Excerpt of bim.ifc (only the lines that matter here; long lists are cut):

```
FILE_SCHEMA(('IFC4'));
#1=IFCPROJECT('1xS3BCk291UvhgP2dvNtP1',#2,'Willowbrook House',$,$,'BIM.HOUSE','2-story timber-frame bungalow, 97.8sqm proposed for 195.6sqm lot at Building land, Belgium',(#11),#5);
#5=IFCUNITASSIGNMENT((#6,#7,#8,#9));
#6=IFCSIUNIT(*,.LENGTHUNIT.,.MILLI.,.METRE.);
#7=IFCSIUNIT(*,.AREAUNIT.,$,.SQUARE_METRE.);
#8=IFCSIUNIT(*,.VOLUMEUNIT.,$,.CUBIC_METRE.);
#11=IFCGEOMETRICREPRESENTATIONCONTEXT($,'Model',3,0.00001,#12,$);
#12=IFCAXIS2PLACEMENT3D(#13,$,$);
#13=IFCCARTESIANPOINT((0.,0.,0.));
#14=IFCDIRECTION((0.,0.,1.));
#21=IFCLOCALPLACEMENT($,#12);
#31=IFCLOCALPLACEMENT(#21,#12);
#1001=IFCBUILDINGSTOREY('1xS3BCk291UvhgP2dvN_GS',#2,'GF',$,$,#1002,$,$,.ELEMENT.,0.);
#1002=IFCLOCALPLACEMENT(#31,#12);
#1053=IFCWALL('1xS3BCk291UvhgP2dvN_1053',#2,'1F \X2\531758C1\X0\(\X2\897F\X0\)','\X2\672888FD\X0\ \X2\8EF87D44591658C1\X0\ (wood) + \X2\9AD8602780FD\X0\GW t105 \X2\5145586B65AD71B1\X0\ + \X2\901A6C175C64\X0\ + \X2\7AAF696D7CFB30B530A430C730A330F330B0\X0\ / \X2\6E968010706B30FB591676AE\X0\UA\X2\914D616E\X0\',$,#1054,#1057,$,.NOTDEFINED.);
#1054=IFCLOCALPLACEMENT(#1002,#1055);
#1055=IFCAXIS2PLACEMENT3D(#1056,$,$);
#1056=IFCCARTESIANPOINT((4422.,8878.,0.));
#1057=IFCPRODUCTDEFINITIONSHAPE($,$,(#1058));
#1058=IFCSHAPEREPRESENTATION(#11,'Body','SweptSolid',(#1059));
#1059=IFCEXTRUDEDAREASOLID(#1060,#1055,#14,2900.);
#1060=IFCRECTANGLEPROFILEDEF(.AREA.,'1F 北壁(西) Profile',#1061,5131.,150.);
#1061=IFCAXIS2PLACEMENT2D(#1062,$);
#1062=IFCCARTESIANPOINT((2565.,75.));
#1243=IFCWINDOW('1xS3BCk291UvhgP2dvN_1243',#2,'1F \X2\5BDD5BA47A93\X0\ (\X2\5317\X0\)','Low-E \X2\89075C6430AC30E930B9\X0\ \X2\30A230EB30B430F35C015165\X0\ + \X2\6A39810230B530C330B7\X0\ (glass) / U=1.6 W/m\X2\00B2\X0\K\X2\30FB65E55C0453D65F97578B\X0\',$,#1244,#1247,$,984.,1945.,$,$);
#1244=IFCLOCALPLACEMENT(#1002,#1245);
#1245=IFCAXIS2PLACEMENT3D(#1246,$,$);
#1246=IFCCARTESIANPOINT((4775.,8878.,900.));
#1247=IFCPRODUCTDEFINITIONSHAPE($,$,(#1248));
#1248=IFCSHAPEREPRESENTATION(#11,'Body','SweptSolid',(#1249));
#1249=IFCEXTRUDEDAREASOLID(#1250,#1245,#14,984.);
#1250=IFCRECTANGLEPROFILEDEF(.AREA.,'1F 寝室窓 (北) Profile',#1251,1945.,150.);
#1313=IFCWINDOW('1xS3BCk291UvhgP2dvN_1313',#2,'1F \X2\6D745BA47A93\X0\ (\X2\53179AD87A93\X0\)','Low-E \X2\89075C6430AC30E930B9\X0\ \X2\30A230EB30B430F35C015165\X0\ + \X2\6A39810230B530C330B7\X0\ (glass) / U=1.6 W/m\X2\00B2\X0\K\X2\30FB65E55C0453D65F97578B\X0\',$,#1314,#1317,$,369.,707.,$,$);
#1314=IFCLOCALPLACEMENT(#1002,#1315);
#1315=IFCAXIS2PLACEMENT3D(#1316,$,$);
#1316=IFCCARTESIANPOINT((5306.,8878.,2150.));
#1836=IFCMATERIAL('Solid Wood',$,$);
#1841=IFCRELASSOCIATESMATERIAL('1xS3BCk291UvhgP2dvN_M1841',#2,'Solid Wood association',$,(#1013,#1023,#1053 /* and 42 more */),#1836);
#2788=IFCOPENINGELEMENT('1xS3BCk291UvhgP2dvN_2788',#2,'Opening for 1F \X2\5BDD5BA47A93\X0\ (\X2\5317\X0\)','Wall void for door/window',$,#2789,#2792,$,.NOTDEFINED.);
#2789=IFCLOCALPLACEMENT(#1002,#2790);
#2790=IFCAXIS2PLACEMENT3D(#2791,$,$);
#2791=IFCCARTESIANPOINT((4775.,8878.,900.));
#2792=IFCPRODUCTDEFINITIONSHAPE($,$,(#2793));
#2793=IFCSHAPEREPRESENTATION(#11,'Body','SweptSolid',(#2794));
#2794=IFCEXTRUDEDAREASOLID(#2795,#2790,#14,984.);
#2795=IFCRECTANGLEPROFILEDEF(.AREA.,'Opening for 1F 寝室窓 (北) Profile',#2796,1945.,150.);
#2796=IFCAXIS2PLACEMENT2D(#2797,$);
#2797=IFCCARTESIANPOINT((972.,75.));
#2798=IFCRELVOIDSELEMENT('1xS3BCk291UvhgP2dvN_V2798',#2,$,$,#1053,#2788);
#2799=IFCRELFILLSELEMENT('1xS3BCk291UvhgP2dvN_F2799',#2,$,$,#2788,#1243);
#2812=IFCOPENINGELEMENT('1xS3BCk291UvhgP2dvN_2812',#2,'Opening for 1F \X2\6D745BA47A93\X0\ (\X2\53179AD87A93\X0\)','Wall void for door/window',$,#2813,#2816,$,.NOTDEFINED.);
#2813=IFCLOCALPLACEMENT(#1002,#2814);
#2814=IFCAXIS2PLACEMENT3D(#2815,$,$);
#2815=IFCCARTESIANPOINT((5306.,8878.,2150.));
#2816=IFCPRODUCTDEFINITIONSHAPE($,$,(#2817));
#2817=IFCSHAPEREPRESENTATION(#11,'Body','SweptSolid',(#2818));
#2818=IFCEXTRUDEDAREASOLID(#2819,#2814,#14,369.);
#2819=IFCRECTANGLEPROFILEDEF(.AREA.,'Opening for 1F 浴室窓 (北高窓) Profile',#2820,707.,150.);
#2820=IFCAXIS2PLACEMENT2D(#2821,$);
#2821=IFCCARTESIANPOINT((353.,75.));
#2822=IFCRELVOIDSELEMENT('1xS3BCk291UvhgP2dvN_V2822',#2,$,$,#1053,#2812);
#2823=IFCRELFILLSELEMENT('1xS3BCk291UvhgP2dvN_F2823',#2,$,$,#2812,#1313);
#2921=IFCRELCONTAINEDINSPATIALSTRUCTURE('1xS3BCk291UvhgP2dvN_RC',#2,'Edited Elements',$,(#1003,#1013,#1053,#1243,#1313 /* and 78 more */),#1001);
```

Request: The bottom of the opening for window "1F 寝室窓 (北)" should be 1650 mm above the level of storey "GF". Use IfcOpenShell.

```python
import numpy as np
import ifcopenshell
import ifcopenshell.api.geometry
import ifcopenshell.geom
import ifcopenshell.util.element
import ifcopenshell.util.placement
import ifcopenshell.util.shape
import ifcopenshell.util.unit

model = ifcopenshell.open("bim.ifc")
unit_scale = ifcopenshell.util.unit.calculate_unit_scale(model)

window = model.by_id(1243)
opening = window.FillsVoids[0].RelatingOpeningElement
storey = ifcopenshell.util.element.get_container(window, ifc_class="IfcBuildingStorey")
level = ifcopenshell.util.placement.get_local_placement(storey.ObjectPlacement)[2, 3]

# The opening's origin need not be at the sill, so measure its lowest point.
shape = ifcopenshell.geom.create_shape(ifcopenshell.geom.settings(), opening)
bottom = ifcopenshell.util.shape.get_shape_bottom_elevation(shape, shape.geometry) / unit_scale
dz = level + 1.65 / unit_scale - bottom

shift = np.array([0.0, 0.0, dz])
# The window is not placed relative to its opening, so move both.
for product in (opening, window):
    matrix = ifcopenshell.util.placement.get_local_placement(product.ObjectPlacement)
    matrix[:3, 3] += shift
    ifcopenshell.api.geometry.edit_object_placement(model, product=product, matrix=matrix, is_si=False)

print(f"moved by {dz * unit_scale:+.3f} m")

model.write("bim-out.ifc")
```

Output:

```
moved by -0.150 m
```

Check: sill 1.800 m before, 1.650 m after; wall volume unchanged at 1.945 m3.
